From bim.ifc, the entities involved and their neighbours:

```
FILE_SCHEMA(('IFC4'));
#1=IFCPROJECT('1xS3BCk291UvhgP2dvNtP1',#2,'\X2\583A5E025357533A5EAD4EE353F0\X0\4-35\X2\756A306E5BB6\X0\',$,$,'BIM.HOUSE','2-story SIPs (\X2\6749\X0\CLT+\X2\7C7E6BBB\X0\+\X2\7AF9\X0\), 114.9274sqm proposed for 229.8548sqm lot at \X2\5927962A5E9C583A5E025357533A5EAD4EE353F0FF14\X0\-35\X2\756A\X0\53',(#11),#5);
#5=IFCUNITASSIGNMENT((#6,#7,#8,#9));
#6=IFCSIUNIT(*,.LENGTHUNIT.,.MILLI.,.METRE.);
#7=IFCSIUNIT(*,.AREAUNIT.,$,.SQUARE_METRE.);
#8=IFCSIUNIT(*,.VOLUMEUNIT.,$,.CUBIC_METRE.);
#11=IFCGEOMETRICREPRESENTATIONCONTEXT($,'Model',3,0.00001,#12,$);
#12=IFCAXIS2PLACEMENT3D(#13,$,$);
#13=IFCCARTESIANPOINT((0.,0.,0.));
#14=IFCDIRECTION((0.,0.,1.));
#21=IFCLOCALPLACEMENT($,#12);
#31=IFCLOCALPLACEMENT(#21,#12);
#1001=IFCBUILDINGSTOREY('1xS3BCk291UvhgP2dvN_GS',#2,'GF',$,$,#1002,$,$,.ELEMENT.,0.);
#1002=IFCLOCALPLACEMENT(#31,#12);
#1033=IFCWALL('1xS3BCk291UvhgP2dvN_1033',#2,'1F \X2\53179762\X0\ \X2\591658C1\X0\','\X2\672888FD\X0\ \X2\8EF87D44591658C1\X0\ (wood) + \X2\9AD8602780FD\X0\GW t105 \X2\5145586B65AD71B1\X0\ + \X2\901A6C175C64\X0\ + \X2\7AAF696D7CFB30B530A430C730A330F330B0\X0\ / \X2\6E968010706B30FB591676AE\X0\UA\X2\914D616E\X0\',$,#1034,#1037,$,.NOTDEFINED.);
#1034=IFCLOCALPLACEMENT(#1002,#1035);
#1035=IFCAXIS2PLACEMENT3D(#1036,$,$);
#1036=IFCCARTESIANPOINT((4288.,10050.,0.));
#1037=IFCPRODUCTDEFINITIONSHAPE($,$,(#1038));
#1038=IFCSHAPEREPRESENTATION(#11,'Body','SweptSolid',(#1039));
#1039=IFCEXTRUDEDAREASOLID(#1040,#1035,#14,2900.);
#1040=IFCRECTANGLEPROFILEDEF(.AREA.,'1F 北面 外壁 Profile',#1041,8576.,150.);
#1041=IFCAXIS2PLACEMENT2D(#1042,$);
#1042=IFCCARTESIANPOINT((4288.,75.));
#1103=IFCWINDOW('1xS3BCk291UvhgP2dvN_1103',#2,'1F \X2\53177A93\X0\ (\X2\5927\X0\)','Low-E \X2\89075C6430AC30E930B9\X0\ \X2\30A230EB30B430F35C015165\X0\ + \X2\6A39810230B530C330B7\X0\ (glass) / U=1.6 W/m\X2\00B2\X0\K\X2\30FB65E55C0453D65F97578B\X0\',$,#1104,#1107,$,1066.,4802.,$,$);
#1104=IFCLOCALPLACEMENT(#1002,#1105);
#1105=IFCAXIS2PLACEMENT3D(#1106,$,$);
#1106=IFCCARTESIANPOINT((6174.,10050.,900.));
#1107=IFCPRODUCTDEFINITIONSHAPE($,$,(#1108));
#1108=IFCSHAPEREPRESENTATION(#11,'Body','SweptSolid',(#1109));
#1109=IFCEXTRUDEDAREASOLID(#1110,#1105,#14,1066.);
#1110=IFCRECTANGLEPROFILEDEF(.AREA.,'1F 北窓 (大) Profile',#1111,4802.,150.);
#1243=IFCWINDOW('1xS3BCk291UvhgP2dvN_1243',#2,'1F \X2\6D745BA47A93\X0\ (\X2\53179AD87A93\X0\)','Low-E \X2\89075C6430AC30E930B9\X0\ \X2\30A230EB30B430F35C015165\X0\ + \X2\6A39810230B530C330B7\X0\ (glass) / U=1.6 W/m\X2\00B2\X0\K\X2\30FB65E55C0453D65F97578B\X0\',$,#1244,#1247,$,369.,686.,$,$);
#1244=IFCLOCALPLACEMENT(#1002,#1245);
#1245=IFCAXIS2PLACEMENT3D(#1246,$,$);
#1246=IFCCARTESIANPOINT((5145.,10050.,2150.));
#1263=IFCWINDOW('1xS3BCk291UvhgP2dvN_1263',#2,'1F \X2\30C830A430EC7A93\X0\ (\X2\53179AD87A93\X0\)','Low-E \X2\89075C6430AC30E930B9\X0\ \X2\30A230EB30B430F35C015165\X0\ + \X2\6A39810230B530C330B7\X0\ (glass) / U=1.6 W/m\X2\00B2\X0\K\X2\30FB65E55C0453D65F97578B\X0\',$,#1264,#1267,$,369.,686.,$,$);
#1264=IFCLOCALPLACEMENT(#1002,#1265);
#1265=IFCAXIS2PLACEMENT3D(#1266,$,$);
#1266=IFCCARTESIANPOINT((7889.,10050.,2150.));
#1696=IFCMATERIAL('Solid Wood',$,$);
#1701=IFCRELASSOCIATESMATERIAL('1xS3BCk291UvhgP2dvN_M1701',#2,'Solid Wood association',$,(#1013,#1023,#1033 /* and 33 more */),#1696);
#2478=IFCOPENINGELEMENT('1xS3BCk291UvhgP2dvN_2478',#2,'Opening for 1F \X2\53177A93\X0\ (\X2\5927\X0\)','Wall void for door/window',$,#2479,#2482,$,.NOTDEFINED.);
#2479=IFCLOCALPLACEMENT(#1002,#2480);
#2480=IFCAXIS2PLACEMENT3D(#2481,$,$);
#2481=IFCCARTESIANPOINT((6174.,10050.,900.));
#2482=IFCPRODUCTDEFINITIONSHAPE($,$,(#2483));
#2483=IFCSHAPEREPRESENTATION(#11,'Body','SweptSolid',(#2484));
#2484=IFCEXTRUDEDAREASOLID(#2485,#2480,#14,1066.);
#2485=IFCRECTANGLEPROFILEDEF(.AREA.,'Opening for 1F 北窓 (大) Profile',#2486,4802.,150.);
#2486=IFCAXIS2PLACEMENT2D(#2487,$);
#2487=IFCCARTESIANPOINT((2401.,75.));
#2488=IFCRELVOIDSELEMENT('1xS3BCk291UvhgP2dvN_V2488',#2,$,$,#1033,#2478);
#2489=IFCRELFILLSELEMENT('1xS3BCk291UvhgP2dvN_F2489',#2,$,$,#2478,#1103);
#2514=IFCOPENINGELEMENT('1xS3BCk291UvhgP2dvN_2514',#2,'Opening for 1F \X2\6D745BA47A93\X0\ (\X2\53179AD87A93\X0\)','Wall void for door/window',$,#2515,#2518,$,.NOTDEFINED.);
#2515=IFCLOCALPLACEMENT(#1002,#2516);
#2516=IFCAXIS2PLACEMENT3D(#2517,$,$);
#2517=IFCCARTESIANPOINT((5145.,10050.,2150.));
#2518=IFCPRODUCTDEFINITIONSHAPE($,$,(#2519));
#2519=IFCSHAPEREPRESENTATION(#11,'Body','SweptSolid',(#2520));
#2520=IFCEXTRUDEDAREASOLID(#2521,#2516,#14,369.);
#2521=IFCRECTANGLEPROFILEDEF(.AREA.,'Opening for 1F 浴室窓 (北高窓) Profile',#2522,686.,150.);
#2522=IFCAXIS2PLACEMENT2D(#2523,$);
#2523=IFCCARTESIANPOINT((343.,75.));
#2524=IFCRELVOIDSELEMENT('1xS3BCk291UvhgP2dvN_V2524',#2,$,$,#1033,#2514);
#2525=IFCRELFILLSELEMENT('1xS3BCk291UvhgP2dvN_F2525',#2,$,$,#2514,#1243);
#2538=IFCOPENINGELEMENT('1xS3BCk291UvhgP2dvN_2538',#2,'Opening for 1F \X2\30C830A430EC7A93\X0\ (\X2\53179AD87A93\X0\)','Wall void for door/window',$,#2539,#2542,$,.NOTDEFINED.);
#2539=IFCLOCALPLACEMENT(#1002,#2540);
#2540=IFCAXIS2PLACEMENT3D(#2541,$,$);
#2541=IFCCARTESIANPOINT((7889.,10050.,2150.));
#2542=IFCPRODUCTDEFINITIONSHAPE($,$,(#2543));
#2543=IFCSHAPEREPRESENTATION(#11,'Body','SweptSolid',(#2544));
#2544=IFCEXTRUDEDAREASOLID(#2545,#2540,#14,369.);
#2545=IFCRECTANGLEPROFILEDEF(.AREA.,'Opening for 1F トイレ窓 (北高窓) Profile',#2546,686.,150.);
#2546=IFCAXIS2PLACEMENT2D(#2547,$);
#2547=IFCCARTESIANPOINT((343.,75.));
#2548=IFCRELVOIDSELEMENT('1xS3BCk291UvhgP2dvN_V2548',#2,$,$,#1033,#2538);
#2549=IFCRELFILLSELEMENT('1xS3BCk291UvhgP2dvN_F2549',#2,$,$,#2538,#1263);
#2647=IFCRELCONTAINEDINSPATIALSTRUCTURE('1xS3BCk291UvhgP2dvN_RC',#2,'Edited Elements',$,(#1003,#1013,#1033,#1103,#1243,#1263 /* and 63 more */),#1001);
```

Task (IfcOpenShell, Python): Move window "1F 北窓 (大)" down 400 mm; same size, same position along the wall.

```python
import numpy as np
import ifcopenshell
import ifcopenshell.api.geometry
import ifcopenshell.util.placement
import ifcopenshell.util.unit

model = ifcopenshell.open("bim.ifc")
unit_scale = ifcopenshell.util.unit.calculate_unit_scale(model)

window = model.by_guid("1xS3BCk291UvhgP2dvN_1103")
opening = window.FillsVoids[0].RelatingOpeningElement
dz = -400.0

shift = np.array([0.0, 0.0, dz])
# The window is not placed relative to its opening, so move both.
for product in (opening, window):
    matrix = ifcopenshell.util.placement.get_local_placement(product.ObjectPlacement)
    matrix[:3, 3] += shift
    ifcopenshell.api.geometry.edit_object_placement(model, product=product, matrix=matrix, is_si=False)

print(f"moved by {dz * unit_scale:+.3f} m")

model.write("bim-out.ifc")
```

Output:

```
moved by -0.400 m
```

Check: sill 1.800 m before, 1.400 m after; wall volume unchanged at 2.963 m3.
